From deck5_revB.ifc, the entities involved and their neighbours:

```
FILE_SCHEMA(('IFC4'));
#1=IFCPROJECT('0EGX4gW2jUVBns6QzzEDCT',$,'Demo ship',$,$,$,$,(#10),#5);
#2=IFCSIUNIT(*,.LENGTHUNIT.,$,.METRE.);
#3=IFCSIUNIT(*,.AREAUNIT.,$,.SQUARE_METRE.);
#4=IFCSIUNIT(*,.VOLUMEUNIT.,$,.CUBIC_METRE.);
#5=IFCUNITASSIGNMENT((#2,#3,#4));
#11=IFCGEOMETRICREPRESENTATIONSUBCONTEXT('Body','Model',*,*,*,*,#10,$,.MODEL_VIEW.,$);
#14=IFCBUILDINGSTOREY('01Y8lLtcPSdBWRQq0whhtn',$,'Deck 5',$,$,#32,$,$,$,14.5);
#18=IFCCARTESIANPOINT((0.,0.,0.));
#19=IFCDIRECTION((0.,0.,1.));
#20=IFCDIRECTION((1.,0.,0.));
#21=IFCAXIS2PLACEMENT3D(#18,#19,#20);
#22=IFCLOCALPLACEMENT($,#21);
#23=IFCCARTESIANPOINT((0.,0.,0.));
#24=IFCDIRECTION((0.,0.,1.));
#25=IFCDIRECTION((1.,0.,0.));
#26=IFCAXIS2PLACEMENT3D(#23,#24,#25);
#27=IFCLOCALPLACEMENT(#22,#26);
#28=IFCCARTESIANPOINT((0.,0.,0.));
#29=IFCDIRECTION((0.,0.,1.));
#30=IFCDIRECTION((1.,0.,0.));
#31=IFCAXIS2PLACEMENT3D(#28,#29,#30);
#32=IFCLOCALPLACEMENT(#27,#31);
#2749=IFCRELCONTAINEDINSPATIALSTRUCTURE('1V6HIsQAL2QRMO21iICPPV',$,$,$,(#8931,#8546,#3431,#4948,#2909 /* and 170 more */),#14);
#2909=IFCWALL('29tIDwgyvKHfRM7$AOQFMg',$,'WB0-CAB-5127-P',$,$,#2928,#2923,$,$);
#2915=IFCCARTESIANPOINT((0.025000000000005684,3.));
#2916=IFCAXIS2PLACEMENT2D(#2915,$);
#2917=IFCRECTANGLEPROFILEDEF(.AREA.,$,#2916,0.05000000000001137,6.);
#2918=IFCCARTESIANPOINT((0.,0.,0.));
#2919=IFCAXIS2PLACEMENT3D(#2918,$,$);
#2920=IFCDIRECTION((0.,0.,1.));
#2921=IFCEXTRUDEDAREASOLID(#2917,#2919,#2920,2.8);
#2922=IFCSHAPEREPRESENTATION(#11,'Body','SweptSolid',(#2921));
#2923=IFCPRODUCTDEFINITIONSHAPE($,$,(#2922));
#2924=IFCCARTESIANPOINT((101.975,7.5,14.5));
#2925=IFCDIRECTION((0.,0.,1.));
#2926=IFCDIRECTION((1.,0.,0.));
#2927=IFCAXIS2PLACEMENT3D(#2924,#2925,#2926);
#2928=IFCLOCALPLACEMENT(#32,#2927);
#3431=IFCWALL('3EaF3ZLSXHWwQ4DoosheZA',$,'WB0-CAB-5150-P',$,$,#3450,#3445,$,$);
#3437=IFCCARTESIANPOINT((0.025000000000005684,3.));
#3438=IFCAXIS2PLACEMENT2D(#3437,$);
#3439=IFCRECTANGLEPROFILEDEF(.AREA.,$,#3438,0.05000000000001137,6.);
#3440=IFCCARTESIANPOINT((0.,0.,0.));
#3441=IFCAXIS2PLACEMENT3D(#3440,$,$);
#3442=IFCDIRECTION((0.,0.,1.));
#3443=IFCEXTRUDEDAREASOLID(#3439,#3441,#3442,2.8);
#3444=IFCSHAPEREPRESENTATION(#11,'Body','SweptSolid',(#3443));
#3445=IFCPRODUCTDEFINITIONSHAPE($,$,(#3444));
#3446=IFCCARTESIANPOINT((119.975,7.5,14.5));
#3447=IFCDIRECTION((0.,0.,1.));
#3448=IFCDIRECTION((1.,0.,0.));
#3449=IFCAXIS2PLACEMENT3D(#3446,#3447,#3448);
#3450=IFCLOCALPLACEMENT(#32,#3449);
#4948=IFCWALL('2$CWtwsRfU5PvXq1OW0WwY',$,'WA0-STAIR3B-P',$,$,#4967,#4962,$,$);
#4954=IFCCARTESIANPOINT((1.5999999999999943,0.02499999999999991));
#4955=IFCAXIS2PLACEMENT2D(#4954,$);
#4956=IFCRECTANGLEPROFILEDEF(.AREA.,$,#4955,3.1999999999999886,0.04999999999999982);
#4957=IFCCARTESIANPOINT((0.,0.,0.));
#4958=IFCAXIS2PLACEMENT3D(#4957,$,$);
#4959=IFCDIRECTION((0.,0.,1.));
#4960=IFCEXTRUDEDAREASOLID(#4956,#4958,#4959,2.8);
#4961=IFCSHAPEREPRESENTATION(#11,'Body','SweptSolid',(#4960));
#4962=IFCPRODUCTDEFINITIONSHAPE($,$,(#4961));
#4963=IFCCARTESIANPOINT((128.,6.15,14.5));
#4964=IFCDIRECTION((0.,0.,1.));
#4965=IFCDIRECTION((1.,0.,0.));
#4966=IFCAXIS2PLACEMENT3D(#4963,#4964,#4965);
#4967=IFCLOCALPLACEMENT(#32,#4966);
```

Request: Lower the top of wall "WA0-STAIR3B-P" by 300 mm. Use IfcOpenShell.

```python
import ifcopenshell
import ifcopenshell.geom
import ifcopenshell.util.representation
import ifcopenshell.util.shape

model = ifcopenshell.open("deck5_revB.ifc")
settings = ifcopenshell.geom.settings()


def volume(element):
    """Net volume in cubic metres, openings subtracted."""
    shape = ifcopenshell.geom.create_shape(settings, element)
    return ifcopenshell.util.shape.get_volume(shape.geometry)


wall = model.by_guid("2$CWtwsRfU5PvXq1OW0WwY")
before = volume(wall)

body = ifcopenshell.util.representation.get_representation(wall, "Model", "Body")
solid = body.Items[0]
old_height = solid.Depth
solid.Depth -= 0.3
after = volume(wall)

print(f"height {old_height:g} -> {solid.Depth:g}, volume {before:.3f} -> {after:.3f} m3")

model.write("deck5_revB_rev.ifc")
```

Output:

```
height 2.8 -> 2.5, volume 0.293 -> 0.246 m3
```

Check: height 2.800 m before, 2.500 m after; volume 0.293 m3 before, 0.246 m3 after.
